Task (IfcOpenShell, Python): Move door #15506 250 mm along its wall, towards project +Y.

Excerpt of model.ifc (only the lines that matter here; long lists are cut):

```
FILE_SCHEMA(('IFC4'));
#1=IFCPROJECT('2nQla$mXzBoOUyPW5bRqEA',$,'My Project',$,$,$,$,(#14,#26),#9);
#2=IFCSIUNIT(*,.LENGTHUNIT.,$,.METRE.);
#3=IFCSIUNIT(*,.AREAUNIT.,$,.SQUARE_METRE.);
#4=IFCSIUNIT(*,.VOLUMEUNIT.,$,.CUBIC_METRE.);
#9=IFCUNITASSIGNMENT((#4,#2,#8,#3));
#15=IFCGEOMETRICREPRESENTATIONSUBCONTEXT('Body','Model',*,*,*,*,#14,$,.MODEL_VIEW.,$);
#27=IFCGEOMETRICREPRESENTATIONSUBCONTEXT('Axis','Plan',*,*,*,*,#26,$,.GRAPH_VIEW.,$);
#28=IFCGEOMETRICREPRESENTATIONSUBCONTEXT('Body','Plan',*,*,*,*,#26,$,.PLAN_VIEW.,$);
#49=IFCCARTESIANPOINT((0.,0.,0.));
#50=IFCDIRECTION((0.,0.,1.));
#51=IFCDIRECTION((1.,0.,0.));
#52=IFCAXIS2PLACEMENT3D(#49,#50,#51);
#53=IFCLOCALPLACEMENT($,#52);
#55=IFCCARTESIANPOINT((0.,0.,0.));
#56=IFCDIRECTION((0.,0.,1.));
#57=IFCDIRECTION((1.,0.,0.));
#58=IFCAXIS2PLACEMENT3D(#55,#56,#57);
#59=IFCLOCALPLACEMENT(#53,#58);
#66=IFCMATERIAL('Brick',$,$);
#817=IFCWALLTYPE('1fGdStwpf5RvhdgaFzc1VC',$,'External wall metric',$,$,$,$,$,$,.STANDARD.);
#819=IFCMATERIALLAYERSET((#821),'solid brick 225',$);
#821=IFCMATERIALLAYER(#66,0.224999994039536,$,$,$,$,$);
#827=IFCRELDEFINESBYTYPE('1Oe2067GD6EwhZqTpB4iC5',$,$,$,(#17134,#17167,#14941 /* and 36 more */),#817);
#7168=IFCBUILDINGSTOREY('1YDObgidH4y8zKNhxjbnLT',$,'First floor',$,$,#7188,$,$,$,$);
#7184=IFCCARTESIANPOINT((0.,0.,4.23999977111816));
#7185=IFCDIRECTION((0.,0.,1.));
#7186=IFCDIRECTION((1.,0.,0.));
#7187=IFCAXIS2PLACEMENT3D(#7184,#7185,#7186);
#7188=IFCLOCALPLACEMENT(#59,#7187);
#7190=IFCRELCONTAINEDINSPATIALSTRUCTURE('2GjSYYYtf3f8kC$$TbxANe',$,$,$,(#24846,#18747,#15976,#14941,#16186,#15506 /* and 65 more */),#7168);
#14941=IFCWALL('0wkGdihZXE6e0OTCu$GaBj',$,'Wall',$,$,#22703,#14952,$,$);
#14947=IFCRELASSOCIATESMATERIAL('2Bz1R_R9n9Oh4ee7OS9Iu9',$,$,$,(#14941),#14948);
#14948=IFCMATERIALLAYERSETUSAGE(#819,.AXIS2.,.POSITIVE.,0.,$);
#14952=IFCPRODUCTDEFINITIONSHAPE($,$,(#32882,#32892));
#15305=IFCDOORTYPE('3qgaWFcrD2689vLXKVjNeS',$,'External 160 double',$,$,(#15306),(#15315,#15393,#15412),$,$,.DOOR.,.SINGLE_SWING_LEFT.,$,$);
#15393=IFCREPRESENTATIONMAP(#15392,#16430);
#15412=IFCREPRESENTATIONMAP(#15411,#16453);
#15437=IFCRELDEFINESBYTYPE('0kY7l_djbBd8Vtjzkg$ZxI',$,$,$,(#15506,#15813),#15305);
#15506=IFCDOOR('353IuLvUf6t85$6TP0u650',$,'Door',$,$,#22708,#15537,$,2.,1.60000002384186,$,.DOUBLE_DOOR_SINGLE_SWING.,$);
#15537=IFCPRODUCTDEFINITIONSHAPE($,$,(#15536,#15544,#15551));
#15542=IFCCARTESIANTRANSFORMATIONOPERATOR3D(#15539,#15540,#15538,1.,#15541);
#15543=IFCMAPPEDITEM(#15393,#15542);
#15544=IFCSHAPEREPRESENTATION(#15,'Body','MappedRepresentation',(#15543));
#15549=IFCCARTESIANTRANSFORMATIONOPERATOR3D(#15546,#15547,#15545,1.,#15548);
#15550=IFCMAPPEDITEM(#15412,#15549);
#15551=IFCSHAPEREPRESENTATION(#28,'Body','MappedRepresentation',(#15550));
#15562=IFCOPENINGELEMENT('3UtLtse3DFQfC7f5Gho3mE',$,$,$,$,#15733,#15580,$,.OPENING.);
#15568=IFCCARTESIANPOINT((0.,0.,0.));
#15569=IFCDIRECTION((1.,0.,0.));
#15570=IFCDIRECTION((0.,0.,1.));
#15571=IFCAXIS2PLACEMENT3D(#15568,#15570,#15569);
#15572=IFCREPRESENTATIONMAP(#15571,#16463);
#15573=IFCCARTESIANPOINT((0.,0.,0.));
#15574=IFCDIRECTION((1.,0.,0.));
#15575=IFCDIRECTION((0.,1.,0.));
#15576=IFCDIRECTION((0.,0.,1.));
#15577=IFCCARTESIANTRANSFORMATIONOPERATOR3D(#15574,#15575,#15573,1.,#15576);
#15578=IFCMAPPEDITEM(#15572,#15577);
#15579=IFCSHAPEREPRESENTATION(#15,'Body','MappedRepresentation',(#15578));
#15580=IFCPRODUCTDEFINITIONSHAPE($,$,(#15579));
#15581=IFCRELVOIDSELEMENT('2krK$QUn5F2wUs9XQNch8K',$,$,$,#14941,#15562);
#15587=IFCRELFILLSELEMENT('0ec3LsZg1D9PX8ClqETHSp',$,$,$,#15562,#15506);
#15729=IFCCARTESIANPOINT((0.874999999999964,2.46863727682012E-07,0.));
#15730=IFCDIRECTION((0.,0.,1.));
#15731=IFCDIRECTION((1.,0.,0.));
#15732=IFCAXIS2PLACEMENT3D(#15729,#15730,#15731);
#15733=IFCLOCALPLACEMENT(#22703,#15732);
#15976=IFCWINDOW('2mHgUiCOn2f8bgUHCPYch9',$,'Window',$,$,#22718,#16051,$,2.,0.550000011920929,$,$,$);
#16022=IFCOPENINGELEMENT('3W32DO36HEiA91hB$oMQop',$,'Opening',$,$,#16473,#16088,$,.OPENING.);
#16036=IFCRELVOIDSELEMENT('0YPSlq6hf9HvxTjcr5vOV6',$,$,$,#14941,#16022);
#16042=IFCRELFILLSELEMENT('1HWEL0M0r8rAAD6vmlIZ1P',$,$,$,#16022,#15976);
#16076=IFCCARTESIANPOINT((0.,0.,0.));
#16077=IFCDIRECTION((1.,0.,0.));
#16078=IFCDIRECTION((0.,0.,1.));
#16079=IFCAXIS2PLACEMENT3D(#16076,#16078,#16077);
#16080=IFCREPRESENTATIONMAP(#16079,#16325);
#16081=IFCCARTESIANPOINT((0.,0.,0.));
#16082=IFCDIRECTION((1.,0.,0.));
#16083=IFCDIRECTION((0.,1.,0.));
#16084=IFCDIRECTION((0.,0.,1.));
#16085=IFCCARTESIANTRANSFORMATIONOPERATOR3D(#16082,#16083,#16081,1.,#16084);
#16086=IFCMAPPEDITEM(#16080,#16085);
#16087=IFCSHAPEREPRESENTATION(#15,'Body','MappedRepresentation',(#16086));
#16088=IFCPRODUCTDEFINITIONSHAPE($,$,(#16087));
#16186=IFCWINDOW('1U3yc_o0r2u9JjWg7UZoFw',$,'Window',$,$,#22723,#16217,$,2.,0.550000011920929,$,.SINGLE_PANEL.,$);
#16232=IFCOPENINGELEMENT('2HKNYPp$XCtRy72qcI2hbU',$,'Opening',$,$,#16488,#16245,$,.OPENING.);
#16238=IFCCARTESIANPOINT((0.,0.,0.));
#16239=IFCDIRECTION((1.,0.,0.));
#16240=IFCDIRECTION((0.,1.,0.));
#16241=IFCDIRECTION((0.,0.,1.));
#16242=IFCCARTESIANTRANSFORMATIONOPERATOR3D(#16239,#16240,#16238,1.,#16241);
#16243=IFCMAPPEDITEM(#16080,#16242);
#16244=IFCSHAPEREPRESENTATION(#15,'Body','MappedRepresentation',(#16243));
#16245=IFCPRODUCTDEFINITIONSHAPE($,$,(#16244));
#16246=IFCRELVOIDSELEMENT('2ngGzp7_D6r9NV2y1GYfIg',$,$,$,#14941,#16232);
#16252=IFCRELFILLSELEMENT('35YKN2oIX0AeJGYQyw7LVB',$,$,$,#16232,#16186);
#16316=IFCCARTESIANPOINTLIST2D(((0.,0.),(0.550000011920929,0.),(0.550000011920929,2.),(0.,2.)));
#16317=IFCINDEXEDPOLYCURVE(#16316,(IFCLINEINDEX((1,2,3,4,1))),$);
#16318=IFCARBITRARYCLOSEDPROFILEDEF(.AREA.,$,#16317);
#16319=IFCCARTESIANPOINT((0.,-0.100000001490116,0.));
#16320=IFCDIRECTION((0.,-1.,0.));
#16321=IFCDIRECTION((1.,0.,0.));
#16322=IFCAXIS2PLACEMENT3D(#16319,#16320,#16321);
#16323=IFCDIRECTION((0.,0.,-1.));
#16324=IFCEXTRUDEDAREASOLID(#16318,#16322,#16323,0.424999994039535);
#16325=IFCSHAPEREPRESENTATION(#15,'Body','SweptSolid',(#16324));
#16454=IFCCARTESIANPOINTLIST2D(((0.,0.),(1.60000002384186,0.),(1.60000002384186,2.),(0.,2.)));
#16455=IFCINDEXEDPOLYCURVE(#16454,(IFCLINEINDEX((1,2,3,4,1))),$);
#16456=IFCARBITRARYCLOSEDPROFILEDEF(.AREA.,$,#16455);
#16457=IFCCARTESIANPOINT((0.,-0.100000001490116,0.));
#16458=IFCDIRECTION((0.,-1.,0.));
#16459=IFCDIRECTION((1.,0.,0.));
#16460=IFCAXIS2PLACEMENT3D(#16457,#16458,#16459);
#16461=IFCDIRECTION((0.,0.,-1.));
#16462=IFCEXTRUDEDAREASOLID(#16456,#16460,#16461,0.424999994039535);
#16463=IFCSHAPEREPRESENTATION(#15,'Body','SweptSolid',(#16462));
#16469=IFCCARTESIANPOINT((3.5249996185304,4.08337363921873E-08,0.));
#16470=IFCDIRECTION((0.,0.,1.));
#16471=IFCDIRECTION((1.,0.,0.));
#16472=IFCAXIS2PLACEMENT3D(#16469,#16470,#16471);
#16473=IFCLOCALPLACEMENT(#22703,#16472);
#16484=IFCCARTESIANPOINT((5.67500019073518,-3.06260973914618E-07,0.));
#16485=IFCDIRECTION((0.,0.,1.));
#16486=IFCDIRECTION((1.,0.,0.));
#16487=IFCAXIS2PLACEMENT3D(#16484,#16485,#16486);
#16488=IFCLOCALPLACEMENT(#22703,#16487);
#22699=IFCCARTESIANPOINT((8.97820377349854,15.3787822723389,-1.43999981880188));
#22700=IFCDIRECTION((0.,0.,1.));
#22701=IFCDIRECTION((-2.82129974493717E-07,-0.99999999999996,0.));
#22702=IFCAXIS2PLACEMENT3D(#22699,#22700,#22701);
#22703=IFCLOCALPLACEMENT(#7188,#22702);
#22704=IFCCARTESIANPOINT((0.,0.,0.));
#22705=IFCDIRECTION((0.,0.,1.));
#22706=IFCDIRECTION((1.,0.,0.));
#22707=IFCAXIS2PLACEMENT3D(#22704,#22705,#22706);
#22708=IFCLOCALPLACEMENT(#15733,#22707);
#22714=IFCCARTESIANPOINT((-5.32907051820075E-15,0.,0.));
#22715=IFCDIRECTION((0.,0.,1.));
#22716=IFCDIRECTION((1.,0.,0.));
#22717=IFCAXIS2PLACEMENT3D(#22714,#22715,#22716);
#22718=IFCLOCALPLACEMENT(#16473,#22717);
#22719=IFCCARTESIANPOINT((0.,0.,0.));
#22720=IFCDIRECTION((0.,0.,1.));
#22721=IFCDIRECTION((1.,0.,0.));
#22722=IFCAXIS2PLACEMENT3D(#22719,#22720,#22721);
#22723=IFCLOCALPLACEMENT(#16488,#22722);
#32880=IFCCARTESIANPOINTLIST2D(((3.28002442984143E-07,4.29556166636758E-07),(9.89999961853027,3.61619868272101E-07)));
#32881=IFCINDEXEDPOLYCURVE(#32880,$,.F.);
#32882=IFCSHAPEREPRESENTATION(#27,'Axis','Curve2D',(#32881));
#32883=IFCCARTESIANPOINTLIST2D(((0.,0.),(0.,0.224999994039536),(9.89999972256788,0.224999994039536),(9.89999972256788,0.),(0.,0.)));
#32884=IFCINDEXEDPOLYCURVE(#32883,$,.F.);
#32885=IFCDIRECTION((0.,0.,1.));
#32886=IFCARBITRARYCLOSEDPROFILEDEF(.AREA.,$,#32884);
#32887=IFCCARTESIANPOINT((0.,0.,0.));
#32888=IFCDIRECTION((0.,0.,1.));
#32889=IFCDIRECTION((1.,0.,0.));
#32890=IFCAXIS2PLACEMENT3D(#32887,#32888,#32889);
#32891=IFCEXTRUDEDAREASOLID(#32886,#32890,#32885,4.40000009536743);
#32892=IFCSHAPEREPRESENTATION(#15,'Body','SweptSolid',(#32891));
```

```python
import ifcopenshell
import ifcopenshell.api.geometry
import ifcopenshell.util.placement
import ifcopenshell.util.unit

model = ifcopenshell.open("model.ifc")
unit_scale = ifcopenshell.util.unit.calculate_unit_scale(model)

door = model.by_guid("353IuLvUf6t85$6TP0u650")
opening = door.FillsVoids[0].RelatingOpeningElement
wall = opening.VoidsElements[0].RelatingBuildingElement

wall_matrix = ifcopenshell.util.placement.get_local_placement(wall.ObjectPlacement)
shift = wall_matrix[:3, 0] * -0.25 / unit_scale
before = ifcopenshell.util.placement.get_local_placement(door.ObjectPlacement)[:3, 3].copy()

# The door is placed relative to its opening, so it follows when the opening moves.
matrix = ifcopenshell.util.placement.get_local_placement(opening.ObjectPlacement)
matrix[:3, 3] += shift
ifcopenshell.api.geometry.edit_object_placement(
    model, product=opening, matrix=matrix, is_si=False, should_transform_children=True
)

after = ifcopenshell.util.placement.get_local_placement(door.ObjectPlacement)[:3, 3]
print("door moved by", (after - before).round(3) + 0.0)

model.write("model_v2.ifc")
```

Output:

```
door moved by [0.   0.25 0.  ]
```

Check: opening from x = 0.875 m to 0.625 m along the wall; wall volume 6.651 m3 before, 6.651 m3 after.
